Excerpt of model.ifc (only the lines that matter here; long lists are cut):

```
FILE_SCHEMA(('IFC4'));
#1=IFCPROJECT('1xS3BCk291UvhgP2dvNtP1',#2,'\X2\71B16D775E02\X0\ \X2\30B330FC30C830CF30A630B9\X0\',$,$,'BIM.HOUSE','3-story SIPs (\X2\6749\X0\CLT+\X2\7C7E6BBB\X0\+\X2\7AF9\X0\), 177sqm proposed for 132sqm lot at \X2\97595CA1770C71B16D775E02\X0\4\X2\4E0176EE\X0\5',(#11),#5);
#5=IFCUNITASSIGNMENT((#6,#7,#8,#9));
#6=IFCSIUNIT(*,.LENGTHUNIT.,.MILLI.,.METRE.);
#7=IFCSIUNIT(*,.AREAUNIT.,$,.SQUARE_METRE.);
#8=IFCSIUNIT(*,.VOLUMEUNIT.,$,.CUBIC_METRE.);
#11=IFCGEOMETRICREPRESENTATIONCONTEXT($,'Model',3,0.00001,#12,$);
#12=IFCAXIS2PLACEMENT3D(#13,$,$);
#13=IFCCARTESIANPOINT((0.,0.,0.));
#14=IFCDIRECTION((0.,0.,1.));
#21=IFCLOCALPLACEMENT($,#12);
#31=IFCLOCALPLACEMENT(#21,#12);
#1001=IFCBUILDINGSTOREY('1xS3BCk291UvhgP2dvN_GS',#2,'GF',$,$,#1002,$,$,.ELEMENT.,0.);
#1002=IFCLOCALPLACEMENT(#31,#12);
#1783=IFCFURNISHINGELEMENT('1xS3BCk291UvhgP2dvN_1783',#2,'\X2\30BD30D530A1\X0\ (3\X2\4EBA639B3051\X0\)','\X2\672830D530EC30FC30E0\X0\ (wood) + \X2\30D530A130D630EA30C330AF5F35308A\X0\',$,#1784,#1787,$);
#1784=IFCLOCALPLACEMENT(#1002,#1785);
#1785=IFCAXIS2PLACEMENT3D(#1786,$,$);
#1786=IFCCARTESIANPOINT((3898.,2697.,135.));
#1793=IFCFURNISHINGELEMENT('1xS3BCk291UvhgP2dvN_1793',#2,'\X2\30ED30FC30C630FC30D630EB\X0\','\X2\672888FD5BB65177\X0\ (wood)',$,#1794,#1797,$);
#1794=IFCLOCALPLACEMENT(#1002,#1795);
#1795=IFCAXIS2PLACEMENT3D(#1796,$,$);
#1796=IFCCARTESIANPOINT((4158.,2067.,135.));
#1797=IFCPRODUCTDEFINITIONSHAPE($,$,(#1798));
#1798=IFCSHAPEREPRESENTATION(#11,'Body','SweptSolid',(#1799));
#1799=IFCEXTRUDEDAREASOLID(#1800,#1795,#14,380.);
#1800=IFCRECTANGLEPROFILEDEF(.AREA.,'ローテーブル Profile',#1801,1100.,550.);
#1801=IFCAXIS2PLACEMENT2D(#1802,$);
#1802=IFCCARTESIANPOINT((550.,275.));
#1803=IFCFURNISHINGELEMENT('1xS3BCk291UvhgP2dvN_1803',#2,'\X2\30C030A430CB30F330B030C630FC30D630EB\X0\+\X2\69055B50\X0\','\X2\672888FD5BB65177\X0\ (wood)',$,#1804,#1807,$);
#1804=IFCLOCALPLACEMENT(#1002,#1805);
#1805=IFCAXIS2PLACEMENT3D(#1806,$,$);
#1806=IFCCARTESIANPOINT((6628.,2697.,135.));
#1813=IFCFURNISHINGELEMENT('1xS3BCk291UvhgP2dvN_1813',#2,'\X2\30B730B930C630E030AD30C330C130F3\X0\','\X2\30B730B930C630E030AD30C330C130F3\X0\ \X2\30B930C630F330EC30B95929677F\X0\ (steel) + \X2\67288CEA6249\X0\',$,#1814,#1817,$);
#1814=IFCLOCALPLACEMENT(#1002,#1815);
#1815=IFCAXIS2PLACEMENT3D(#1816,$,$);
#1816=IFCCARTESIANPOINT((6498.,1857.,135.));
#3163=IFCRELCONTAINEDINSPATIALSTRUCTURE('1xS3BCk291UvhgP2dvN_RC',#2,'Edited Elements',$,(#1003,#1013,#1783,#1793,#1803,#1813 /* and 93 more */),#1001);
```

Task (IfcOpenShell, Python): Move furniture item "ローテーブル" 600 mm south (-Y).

```python
import ifcopenshell
import ifcopenshell.api.geometry
import ifcopenshell.util.placement
import ifcopenshell.util.unit

model = ifcopenshell.open("model.ifc")
unit_scale = ifcopenshell.util.unit.calculate_unit_scale(model)

item = model.by_guid("1xS3BCk291UvhgP2dvN_1793")
matrix = ifcopenshell.util.placement.get_local_placement(item.ObjectPlacement)
matrix[1, 3] -= 0.6 / unit_scale
ifcopenshell.api.geometry.edit_object_placement(model, product=item, matrix=matrix, is_si=False)

print(ifcopenshell.util.placement.get_local_placement(item.ObjectPlacement).round(3) + 0.0)

model.write("model_edited.ifc")
```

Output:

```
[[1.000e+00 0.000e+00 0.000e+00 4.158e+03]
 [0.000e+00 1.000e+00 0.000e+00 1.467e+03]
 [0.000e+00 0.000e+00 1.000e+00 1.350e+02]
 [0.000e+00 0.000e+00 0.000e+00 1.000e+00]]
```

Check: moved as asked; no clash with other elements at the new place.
